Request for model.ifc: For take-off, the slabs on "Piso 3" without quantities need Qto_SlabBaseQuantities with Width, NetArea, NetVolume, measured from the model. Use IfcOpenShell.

First a look at what the model holds.

```python
import ifcopenshell
import ifcopenshell.util.element
import ifcopenshell.util.unit

model = ifcopenshell.open("model.ifc")
print(model.schema)
for unit_type in ("LENGTHUNIT", "AREAUNIT", "VOLUMEUNIT"):
    print(unit_type, ifcopenshell.util.unit.calculate_unit_scale(model, unit_type))
storey = next(s for s in model.by_type("IfcBuildingStorey") if s.Name == "Piso 3")
slabs = [e for e in ifcopenshell.util.element.get_decomposition(storey) if e.is_a("IfcSlab")]
for e in sorted(slabs, key=lambda e: e.id()):
    print(e.id(), e.is_a(), e.Name, list(ifcopenshell.util.element.get_psets(e, qtos_only=True)), sep=" | ")
```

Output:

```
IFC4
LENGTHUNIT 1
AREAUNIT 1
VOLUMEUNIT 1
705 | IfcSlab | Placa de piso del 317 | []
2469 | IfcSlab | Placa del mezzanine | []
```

```python
import ifcopenshell
import ifcopenshell.api.pset
import ifcopenshell.geom
import ifcopenshell.util.element
import ifcopenshell.util.shape
import ifcopenshell.util.unit

model = ifcopenshell.open("model.ifc")
unit_scale = ifcopenshell.util.unit.calculate_unit_scale(model)
area_scale = ifcopenshell.util.unit.calculate_unit_scale(model, "AREAUNIT")
volume_scale = ifcopenshell.util.unit.calculate_unit_scale(model, "VOLUMEUNIT")
settings = ifcopenshell.geom.settings()

storey = next(s for s in model.by_type("IfcBuildingStorey") if s.Name == "Piso 3")
slabs = [e for e in ifcopenshell.util.element.get_decomposition(storey) if e.is_a("IfcSlab")]

for e in sorted(slabs, key=lambda e: e.id()):
    if ifcopenshell.util.element.get_psets(e, qtos_only=True, should_inherit=False):
        continue
    # Geometry comes back in metres, in the element's own axes.
    shape = ifcopenshell.geom.create_shape(settings, e)
    values = {
        "Width": ifcopenshell.util.shape.get_z(shape.geometry) / unit_scale,
        "NetArea": ifcopenshell.util.shape.get_footprint_area(shape.geometry) / area_scale,
        "NetVolume": ifcopenshell.util.shape.get_volume(shape.geometry) / volume_scale,
    }
    qto = ifcopenshell.api.pset.add_qto(model, product=e, name="Qto_SlabBaseQuantities")
    ifcopenshell.api.pset.edit_qto(model, qto=qto, properties=values)
    print(e.id(), {k: round(v, 3) for k, v in values.items()})

model.write("model_rev.ifc")
```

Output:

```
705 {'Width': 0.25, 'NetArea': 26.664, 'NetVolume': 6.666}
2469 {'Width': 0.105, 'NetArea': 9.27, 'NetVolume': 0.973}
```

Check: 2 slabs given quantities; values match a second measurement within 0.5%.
